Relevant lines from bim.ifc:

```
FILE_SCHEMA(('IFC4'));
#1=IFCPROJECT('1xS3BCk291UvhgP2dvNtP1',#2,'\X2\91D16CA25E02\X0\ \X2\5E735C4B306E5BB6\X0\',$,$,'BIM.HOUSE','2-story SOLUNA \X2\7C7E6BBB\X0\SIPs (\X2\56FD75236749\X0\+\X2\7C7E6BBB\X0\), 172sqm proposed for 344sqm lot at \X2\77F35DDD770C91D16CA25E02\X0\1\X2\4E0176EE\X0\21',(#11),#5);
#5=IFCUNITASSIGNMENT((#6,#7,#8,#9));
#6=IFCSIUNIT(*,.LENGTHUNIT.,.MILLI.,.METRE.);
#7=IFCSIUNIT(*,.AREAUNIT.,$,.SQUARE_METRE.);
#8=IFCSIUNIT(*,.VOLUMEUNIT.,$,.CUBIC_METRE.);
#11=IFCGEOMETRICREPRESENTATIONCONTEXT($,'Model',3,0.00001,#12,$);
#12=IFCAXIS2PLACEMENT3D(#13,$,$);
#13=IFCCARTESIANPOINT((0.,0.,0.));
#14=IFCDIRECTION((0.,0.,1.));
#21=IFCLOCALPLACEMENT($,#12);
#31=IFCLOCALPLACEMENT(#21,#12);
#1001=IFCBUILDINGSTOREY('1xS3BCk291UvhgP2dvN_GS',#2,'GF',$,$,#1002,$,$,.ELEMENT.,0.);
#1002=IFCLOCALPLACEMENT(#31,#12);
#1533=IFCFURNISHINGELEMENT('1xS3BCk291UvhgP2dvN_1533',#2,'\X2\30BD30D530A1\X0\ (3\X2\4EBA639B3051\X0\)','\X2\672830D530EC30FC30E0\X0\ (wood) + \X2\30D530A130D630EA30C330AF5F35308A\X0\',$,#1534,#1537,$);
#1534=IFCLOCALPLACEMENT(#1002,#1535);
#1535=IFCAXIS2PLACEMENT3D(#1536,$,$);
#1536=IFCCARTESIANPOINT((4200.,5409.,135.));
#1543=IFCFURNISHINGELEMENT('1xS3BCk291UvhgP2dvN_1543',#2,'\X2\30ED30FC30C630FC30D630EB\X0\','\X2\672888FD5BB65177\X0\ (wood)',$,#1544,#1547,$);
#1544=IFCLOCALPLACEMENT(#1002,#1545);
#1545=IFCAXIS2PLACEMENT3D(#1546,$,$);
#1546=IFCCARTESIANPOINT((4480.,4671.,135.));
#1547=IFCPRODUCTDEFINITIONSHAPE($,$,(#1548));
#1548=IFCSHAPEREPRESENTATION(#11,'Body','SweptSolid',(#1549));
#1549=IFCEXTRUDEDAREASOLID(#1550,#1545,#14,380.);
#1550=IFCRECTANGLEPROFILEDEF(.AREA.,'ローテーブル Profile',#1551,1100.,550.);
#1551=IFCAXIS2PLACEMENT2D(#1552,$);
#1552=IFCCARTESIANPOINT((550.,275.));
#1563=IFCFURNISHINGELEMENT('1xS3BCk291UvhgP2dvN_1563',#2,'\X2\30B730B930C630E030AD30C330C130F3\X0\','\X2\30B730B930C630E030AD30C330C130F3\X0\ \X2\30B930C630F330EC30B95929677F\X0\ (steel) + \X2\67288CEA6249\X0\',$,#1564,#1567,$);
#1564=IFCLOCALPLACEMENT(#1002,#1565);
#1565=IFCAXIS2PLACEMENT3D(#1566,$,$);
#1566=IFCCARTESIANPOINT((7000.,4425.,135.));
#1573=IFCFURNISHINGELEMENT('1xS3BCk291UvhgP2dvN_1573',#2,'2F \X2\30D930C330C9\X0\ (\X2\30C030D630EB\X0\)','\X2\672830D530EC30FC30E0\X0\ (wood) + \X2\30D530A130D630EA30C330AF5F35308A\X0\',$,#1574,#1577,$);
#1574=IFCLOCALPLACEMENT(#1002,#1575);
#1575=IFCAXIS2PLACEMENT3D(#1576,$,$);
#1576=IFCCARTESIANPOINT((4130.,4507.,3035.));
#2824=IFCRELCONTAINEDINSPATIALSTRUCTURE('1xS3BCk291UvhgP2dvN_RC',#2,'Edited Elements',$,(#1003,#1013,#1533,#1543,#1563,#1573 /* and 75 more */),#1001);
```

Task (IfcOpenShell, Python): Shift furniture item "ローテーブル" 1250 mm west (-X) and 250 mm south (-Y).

```python
import ifcopenshell
import ifcopenshell.api.geometry
import ifcopenshell.util.placement
import ifcopenshell.util.unit

model = ifcopenshell.open("bim.ifc")
unit_scale = ifcopenshell.util.unit.calculate_unit_scale(model)

item = model.by_id(1543)
matrix = ifcopenshell.util.placement.get_local_placement(item.ObjectPlacement)
matrix[0, 3] -= 1.25 / unit_scale
matrix[1, 3] -= 0.25 / unit_scale
ifcopenshell.api.geometry.edit_object_placement(model, product=item, matrix=matrix, is_si=False)

print(ifcopenshell.util.placement.get_local_placement(item.ObjectPlacement).round(3) + 0.0)

model.write("bim_v2.ifc")
```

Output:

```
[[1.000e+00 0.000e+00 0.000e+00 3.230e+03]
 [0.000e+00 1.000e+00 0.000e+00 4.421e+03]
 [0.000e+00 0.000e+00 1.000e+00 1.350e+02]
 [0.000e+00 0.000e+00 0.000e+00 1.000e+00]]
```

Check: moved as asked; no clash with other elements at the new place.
